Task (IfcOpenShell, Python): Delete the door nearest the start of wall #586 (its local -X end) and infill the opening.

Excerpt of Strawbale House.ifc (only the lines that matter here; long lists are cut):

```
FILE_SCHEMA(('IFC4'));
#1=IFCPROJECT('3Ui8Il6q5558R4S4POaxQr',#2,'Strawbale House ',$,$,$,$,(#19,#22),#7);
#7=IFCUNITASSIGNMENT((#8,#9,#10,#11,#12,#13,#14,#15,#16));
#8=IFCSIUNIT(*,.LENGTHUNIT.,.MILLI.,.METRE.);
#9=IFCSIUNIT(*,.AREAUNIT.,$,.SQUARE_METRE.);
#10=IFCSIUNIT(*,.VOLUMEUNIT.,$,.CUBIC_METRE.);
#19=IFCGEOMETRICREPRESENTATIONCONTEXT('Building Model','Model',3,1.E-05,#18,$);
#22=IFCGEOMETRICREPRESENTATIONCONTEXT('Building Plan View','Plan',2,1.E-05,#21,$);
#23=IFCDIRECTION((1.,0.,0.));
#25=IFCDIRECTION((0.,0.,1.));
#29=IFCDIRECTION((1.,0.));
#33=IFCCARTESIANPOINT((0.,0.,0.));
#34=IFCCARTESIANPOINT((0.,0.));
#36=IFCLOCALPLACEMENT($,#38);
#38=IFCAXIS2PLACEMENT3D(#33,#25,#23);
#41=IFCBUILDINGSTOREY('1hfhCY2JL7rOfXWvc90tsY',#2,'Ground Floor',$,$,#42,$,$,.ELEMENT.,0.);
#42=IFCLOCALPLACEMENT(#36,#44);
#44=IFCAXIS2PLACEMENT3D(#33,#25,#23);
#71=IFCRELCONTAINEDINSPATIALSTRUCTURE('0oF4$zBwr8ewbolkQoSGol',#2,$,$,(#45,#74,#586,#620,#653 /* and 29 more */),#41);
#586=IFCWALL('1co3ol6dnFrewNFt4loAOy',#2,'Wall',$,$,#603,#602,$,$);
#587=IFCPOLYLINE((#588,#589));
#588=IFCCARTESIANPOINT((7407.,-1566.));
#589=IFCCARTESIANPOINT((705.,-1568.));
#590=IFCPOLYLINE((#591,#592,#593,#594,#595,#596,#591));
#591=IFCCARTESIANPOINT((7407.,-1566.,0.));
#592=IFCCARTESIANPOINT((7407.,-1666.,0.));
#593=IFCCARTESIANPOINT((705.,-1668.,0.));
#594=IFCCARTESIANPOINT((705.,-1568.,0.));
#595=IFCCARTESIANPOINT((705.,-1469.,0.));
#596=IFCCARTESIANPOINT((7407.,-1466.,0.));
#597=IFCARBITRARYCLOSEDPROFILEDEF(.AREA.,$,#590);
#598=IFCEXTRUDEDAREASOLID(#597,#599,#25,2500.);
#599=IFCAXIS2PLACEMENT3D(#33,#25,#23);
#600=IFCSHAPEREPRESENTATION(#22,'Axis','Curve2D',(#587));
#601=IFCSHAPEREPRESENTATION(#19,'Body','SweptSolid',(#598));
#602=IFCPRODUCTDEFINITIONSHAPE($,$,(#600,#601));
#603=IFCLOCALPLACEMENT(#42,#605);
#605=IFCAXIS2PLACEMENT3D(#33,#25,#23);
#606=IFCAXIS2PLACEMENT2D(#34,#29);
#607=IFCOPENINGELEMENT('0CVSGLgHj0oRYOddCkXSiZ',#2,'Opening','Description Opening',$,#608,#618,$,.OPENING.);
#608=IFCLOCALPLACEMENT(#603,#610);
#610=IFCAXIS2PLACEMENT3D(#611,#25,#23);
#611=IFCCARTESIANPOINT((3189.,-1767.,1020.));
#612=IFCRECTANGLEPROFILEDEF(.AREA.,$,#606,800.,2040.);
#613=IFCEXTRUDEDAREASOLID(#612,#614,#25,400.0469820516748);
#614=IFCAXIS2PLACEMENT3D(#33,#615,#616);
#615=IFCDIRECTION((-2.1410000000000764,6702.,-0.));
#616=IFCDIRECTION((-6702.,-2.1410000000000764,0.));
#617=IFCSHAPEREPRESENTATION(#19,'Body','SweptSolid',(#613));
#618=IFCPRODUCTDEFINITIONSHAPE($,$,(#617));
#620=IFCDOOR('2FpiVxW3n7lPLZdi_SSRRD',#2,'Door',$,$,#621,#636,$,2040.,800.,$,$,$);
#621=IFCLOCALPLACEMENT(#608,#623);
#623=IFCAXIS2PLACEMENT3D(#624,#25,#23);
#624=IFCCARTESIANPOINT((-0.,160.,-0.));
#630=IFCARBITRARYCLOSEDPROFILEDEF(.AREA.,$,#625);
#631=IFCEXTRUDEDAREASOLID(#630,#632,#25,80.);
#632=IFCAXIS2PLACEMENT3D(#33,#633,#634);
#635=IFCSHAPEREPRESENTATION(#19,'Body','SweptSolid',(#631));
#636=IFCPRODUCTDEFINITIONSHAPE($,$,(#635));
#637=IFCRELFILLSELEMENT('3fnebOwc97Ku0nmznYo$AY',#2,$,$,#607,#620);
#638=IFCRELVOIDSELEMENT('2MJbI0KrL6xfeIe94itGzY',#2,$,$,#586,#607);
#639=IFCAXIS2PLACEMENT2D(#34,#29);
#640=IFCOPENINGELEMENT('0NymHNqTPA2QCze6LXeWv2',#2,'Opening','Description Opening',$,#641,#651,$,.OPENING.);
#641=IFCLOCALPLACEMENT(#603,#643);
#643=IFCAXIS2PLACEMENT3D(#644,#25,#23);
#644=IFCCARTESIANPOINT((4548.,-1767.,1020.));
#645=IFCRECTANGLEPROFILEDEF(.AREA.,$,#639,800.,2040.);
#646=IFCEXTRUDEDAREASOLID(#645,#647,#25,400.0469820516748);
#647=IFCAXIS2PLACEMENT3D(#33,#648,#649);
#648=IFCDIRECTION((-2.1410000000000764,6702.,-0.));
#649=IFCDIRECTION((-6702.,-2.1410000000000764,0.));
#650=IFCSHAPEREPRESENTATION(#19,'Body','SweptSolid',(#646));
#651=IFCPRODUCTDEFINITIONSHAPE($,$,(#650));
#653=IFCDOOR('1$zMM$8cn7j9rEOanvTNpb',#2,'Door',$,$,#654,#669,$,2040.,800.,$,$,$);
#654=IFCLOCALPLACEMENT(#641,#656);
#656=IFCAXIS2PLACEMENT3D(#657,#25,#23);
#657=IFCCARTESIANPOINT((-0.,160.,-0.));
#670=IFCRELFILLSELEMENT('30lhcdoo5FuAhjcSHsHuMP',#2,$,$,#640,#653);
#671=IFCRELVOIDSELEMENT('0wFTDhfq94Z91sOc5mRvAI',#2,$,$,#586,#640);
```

```python
import ifcopenshell
import ifcopenshell.api.feature
import ifcopenshell.api.root
import ifcopenshell.geom
import ifcopenshell.util.shape

model = ifcopenshell.open("Strawbale House.ifc")
settings = ifcopenshell.geom.settings()


def volume(element):
    """Net volume in cubic metres, openings subtracted."""
    shape = ifcopenshell.geom.create_shape(settings, element)
    return ifcopenshell.util.shape.get_volume(shape.geometry)


door = model.by_id(620)
opening = door.FillsVoids[0].RelatingOpeningElement
wall = opening.VoidsElements[0].RelatingBuildingElement
before = volume(wall)

ifcopenshell.api.root.remove_product(model, product=door)
ifcopenshell.api.feature.remove_feature(model, feature=opening)

after = volume(wall)

print(f"wall volume {before:.3f} -> {after:.3f} m3")

model.write("Strawbale House_rev.ifc")
```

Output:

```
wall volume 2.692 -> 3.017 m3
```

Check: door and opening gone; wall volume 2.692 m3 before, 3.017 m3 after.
